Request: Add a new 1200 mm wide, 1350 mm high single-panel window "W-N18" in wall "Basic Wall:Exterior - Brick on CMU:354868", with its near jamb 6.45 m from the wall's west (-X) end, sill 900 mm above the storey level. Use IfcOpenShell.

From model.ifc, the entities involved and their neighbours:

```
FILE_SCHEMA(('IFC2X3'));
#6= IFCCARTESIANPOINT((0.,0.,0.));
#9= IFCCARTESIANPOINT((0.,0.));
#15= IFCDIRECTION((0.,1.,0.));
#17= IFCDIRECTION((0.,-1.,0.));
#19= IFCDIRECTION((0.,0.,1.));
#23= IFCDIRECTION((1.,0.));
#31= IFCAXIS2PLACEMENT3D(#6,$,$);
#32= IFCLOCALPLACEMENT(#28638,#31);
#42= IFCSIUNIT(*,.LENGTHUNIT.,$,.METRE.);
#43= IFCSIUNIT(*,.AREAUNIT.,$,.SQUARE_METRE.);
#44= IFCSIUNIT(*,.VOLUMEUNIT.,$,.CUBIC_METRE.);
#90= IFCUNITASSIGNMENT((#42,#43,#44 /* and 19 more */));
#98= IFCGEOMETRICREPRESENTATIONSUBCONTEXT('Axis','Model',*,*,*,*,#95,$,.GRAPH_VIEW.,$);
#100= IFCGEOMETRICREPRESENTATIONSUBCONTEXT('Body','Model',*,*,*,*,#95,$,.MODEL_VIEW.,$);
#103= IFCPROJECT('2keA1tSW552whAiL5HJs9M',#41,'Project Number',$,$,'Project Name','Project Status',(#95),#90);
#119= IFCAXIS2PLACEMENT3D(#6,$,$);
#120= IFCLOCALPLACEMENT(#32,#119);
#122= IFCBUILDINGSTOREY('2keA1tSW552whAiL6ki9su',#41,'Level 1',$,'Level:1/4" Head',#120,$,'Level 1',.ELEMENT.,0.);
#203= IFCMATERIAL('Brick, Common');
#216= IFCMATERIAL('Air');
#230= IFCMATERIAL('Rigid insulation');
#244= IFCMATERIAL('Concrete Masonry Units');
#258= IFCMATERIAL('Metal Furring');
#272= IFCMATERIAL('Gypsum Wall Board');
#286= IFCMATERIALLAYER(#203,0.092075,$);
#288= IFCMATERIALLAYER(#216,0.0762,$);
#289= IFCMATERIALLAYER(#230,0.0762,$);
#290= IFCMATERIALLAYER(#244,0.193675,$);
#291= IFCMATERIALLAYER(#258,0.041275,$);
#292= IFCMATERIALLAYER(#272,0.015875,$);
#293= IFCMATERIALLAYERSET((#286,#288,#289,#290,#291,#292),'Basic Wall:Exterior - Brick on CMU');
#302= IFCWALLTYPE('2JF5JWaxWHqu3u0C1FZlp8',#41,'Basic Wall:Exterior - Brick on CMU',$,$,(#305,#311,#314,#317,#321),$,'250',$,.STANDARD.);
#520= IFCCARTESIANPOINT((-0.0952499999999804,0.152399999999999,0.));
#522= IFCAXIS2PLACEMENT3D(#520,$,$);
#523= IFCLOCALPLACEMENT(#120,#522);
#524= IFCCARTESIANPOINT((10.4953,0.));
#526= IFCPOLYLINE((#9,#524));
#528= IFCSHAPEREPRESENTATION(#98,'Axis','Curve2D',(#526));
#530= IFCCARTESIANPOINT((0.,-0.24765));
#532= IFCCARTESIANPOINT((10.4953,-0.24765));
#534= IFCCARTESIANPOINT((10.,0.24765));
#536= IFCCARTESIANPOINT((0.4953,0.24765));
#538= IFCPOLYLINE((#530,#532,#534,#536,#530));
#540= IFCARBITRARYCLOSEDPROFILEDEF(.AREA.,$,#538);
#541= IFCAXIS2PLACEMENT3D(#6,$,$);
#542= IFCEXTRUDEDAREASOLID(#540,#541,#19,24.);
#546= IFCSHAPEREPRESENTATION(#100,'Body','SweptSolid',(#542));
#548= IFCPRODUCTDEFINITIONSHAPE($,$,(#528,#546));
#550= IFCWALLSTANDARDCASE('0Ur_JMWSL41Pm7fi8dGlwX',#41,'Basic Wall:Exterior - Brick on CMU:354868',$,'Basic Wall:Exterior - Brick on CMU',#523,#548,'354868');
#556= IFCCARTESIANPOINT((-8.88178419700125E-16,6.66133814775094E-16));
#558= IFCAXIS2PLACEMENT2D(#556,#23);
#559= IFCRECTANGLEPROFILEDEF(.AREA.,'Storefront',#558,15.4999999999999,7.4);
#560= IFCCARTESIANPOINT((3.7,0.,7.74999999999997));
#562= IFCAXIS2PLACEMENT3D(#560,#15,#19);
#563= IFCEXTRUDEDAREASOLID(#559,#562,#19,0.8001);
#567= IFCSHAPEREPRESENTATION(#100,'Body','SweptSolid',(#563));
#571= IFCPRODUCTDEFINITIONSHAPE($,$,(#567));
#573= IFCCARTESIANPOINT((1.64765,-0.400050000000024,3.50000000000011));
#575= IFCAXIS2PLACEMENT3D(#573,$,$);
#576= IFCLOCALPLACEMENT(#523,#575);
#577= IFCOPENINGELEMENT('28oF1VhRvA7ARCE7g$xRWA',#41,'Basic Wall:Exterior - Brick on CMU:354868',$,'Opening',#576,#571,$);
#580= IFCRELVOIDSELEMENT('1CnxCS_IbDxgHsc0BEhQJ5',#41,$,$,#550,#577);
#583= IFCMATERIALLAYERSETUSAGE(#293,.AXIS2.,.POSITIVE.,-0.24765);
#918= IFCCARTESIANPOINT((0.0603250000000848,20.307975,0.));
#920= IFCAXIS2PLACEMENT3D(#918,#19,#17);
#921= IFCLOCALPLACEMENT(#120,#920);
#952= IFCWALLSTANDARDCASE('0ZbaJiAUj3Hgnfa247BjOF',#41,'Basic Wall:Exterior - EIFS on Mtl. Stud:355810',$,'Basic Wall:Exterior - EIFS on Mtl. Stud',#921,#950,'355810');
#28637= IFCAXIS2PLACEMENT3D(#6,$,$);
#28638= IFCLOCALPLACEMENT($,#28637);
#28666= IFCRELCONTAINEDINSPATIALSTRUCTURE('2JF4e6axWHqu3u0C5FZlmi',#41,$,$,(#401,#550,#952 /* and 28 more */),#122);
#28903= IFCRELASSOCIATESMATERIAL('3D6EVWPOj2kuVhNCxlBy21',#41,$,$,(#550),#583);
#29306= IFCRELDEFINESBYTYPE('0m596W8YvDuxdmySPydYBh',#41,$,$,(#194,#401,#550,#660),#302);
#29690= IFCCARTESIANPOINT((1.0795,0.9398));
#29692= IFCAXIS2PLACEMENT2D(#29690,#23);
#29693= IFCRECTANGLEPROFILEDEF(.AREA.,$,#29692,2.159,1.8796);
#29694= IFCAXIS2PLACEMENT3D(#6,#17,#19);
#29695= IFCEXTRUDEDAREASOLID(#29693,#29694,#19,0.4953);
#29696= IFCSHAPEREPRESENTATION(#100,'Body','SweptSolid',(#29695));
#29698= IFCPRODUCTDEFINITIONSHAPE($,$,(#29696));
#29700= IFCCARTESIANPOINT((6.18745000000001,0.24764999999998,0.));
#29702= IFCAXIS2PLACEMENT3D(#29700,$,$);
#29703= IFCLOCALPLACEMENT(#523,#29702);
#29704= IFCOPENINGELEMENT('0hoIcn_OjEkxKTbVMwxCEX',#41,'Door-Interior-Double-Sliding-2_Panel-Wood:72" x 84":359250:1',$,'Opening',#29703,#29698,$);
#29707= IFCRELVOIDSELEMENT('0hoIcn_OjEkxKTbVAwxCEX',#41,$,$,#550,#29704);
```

```python
import numpy as np
import ifcopenshell
import ifcopenshell.api.feature
import ifcopenshell.api.geometry
import ifcopenshell.api.root
import ifcopenshell.api.spatial
import ifcopenshell.api.type
import ifcopenshell.geom
import ifcopenshell.util.element
import ifcopenshell.util.placement
import ifcopenshell.util.representation
import ifcopenshell.util.shape
import ifcopenshell.util.unit

model = ifcopenshell.open("model.ifc")
unit_scale = ifcopenshell.util.unit.calculate_unit_scale(model)
settings = ifcopenshell.geom.settings()


def volume(element):
    """Net volume in cubic metres, openings subtracted."""
    shape = ifcopenshell.geom.create_shape(settings, element)
    return ifcopenshell.util.shape.get_volume(shape.geometry)


wall = model.by_guid("0Ur_JMWSL41Pm7fi8dGlwX")
storey = ifcopenshell.util.element.get_container(wall, ifc_class="IfcBuildingStorey")
context = ifcopenshell.util.representation.get_context(model, "Model", "Body", "MODEL_VIEW")
before = volume(wall)

width, height, from_end, sill = 1.2, 1.35, 6.45, 0.9  # metres

# The wall runs along its own X axis, and the end named is its -X end.
wall_shape = ifcopenshell.geom.create_shape(settings, wall)
x, y, z = ifcopenshell.util.shape.get_vertices(wall_shape.geometry).T
start = x.min() + from_end
face, thickness = float(y.min()), float(y.max() - y.min())
wall_matrix = ifcopenshell.util.placement.get_local_placement(wall.ObjectPlacement)
level = ifcopenshell.util.placement.get_local_placement(storey.ObjectPlacement)[2, 3]


def in_wall(x, y):
    """Placement at x, y metres in the wall's axes, at sill height."""
    matrix = wall_matrix.copy()
    matrix[:, 3] = wall_matrix @ np.array([x / unit_scale, y / unit_scale, 0.0, 1.0])
    matrix[2, 3] = level + sill / unit_scale
    return matrix


# Opening: a box that overshoots both wall faces by 50 mm.
opening = ifcopenshell.api.root.create_entity(model, ifc_class="IfcOpeningElement")
box = ifcopenshell.api.geometry.add_wall_representation(
    model, context=context, length=width, height=height, thickness=thickness + 0.1
)
ifcopenshell.api.geometry.assign_representation(model, product=opening, representation=box)
ifcopenshell.api.geometry.edit_object_placement(model, product=opening, matrix=in_wall(start, face - 0.05), is_si=False)
ifcopenshell.api.feature.add_feature(model, feature=opening, element=wall)

window = ifcopenshell.api.root.create_entity(model, ifc_class="IfcWindow", name="W-N18")
window.OverallWidth, window.OverallHeight = width / unit_scale, height / unit_scale
body = ifcopenshell.api.geometry.add_window_representation(
    model,
    context=context,
    overall_width=window.OverallWidth,
    overall_height=window.OverallHeight,
    partition_type="SINGLE_PANEL",
)
ifcopenshell.api.geometry.assign_representation(model, product=window, representation=body)
ifcopenshell.api.spatial.assign_container(model, products=[window], relating_structure=storey)
fills = ifcopenshell.api.feature.add_filling(model, opening=opening, element=window)
fills.OwnerHistory = window.OwnerHistory  # required in IFC2X3

# IFC2X3 keeps the operation on the window style.
style = ifcopenshell.api.root.create_entity(model, ifc_class="IfcWindowStyle", name="W-N18")
style.OperationType, style.ConstructionType = "SINGLE_PANEL", "NOTDEFINED"
style.ParameterTakesPrecedence = style.Sizeable = False
ifcopenshell.api.type.assign_type(model, related_objects=[window], relating_type=style)

# Centre the window in the wall's thickness.
ifcopenshell.api.geometry.edit_object_placement(model, product=window, matrix=in_wall(start, face), is_si=False)
window_shape = ifcopenshell.geom.create_shape(settings, window)
depth = ifcopenshell.util.shape.get_vertices(window_shape.geometry)[:, 1]
offset = face + thickness / 2 - (depth.min() + depth.max()) / 2
ifcopenshell.api.geometry.edit_object_placement(model, product=window, matrix=in_wall(start, offset), is_si=False)

after = volume(wall)

print(f"wall volume {before:.3f} -> {after:.3f} m3")

model.write("model_edited.ifc")
```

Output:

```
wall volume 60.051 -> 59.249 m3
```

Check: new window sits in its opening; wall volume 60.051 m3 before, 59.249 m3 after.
